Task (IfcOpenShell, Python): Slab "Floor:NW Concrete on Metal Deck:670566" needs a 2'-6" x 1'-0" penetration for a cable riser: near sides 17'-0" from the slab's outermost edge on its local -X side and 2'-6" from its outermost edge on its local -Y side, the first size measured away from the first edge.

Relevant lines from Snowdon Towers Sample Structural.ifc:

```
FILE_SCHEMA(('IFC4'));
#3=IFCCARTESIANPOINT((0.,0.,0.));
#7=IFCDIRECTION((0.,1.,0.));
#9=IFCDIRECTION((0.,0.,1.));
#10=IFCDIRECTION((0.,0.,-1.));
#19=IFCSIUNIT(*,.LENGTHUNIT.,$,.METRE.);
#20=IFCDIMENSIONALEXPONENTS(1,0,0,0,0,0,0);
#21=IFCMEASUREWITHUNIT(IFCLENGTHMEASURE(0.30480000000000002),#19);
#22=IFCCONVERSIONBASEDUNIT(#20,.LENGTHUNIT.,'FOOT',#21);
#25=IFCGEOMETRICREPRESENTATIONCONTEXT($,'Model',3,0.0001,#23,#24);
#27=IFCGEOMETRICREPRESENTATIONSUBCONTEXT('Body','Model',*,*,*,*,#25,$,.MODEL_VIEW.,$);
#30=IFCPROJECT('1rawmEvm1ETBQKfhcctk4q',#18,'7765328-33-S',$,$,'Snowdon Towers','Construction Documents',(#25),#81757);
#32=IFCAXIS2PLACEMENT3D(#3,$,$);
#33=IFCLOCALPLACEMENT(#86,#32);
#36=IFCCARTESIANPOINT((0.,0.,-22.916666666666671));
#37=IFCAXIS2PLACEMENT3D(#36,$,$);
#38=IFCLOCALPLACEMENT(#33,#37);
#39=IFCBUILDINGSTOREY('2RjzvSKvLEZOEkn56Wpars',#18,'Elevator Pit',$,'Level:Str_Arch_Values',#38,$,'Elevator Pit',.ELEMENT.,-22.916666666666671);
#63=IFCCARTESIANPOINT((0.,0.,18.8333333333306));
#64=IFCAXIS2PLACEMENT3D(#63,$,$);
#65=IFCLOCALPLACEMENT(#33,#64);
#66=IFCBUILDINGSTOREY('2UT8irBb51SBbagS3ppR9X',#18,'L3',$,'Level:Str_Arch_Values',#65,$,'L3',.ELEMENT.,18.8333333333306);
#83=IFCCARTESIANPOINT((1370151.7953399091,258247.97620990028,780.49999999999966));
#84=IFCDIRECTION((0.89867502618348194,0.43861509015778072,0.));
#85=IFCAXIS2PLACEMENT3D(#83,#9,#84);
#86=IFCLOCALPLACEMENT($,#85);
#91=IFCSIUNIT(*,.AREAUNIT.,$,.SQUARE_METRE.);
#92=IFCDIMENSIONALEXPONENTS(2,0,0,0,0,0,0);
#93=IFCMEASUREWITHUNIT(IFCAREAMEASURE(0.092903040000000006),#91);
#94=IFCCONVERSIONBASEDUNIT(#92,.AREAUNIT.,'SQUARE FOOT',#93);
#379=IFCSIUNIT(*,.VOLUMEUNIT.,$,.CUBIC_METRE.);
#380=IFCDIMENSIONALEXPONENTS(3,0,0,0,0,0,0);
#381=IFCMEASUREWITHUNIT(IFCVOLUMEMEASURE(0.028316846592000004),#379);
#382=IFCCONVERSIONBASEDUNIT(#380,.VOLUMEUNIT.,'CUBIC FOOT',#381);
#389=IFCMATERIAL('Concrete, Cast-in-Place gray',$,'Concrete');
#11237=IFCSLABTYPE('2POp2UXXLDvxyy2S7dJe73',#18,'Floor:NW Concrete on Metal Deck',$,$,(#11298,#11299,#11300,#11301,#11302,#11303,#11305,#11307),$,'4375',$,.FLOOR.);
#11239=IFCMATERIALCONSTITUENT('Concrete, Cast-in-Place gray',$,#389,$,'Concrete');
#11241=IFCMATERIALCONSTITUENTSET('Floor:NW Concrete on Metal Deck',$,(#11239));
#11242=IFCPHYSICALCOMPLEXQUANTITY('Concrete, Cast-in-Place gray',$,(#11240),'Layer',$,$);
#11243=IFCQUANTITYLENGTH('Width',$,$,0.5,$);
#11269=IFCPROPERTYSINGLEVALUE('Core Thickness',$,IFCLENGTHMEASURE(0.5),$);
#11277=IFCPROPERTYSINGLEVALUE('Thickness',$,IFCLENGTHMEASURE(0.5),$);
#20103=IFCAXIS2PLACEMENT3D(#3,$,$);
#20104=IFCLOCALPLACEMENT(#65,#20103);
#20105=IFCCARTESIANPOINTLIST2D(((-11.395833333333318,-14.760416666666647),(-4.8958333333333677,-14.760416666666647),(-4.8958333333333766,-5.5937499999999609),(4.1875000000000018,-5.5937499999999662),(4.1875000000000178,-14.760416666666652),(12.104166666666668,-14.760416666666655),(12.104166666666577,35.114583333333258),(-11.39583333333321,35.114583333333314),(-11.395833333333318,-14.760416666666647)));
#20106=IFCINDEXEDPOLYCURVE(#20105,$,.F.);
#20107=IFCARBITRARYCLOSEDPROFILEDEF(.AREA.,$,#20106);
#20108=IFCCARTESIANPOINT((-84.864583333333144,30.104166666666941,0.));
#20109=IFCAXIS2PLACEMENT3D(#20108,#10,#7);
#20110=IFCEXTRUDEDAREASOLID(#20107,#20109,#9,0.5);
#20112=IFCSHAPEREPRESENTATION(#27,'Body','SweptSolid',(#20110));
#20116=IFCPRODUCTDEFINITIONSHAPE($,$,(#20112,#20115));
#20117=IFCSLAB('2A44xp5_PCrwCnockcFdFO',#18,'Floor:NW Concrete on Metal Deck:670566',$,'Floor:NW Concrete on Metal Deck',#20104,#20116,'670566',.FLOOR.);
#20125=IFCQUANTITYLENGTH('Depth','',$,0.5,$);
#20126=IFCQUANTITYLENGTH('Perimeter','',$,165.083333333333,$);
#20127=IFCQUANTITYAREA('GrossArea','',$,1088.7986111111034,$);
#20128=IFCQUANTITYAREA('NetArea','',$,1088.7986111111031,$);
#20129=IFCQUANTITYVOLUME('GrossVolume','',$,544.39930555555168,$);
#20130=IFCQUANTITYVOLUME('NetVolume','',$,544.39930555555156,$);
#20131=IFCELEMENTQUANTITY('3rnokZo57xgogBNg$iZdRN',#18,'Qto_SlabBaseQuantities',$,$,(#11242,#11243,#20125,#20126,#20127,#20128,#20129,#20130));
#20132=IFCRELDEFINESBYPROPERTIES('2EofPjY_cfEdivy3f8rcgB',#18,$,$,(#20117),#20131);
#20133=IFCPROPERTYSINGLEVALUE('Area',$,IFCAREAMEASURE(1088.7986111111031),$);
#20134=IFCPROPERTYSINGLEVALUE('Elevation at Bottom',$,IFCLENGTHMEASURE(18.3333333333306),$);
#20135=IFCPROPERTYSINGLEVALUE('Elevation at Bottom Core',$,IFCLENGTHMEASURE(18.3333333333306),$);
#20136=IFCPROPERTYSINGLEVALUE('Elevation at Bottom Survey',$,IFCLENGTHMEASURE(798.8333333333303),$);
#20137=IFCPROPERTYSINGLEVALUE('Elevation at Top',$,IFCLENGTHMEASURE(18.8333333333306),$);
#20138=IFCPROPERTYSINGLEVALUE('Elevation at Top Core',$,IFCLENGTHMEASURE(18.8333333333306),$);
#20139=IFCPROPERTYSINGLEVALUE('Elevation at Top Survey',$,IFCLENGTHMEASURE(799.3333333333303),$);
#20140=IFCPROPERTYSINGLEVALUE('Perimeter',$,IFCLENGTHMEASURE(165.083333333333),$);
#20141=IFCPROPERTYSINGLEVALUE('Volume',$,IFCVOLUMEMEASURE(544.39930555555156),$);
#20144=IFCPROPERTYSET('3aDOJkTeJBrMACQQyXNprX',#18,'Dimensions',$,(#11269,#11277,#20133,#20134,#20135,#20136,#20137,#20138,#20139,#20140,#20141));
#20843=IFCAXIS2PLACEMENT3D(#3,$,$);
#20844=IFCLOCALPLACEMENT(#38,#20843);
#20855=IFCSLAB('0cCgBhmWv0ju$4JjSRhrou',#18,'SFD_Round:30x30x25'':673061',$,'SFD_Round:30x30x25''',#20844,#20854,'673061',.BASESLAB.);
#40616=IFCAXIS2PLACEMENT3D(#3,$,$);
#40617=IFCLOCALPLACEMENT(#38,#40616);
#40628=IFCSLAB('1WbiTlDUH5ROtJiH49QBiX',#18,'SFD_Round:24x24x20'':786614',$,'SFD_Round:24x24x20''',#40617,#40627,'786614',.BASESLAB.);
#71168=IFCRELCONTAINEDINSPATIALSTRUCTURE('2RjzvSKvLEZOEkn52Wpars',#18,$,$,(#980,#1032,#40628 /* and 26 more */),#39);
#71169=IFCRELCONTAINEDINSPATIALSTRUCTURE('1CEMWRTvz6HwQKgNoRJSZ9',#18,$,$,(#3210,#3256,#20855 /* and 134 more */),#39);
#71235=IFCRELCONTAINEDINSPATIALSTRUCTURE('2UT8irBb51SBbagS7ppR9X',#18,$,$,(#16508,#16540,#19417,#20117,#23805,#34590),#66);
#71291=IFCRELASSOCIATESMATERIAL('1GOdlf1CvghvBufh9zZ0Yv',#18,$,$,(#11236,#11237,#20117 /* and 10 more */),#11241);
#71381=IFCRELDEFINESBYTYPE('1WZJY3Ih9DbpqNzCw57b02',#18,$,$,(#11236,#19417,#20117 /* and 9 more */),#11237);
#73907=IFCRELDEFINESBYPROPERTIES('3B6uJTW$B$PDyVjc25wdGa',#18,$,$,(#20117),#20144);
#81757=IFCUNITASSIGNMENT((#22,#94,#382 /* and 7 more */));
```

```python
import numpy as np
import ifcopenshell
import ifcopenshell.api.feature
import ifcopenshell.api.geometry
import ifcopenshell.api.pset
import ifcopenshell.api.root
import ifcopenshell.geom
import ifcopenshell.util.element
import ifcopenshell.util.placement
import ifcopenshell.util.representation
import ifcopenshell.util.shape
import ifcopenshell.util.unit

model = ifcopenshell.open("Snowdon Towers Sample Structural.ifc")
unit_scale = ifcopenshell.util.unit.calculate_unit_scale(model)
area_scale = ifcopenshell.util.unit.calculate_unit_scale(model, "AREAUNIT")
volume_scale = ifcopenshell.util.unit.calculate_unit_scale(model, "VOLUMEUNIT")
settings = ifcopenshell.geom.settings()


def volume(element):
    """Net volume in cubic metres, openings subtracted."""
    shape = ifcopenshell.geom.create_shape(settings, element)
    return ifcopenshell.util.shape.get_volume(shape.geometry)


slab = model.by_guid("2A44xp5_PCrwCnockcFdFO")
before = volume(slab)

# Extent in the slab's own axes, in metres. The edges named are its -X and -Y sides.
slab_shape = ifcopenshell.geom.create_shape(settings, slab)
vertices = ifcopenshell.util.shape.get_vertices(slab_shape.geometry)
x_min, y_min, bottom = vertices.min(axis=0)
top = vertices[:, 2].max()

opening = ifcopenshell.api.root.create_entity(model, ifc_class="IfcOpeningElement", name="Cable riser opening", predefined_type="OPENING")
context = ifcopenshell.util.representation.get_context(model, "Model", "Body", "MODEL_VIEW")
width, depth = 0.762, 0.3048
outline = [(0.0, 0.0), (width, 0.0), (width, depth), (0.0, depth), (0.0, 0.0)]
# Overshoot both faces by 50 mm so the cut is clean.
shape = ifcopenshell.api.geometry.add_slab_representation(
    model, context=context, depth=top - bottom + 0.1, polyline=outline
)
ifcopenshell.api.geometry.assign_representation(model, product=opening, representation=shape)

matrix = ifcopenshell.util.placement.get_local_placement(slab.ObjectPlacement)
matrix[:, 3] = matrix @ np.append(np.array([x_min + 5.1816, y_min + 0.762, bottom - 0.05]) / unit_scale, 1.0)
ifcopenshell.api.geometry.edit_object_placement(model, product=opening, matrix=matrix, is_si=False)
ifcopenshell.api.feature.add_feature(model, feature=opening, element=slab)

after = volume(slab)

# Update the slab's stored quantities.
qto = model.by_id(ifcopenshell.util.element.get_pset(slab, "Qto_SlabBaseQuantities", should_inherit=False)["id"])
ifcopenshell.api.pset.edit_qto(model, qto=qto, properties={
    "NetArea": after / (top - bottom) / area_scale,
    "NetVolume": after / volume_scale,
})
pset = model.by_id(ifcopenshell.util.element.get_pset(slab, "Dimensions", should_inherit=False)["id"])
ifcopenshell.api.pset.edit_pset(model, pset=pset, properties={
    "Area": model.create_entity("IfcAreaMeasure", after / (top - bottom) / area_scale),
    "Volume": model.create_entity("IfcVolumeMeasure", after / volume_scale),
})

print(f"slab volume {before:.3f} -> {after:.3f} m3")

model.write("Snowdon Towers Sample Structural_rev.ifc")
```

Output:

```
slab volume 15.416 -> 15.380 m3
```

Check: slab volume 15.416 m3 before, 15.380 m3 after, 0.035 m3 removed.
